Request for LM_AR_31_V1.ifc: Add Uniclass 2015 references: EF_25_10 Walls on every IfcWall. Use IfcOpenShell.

First a look at what the model holds.

```python
import ifcopenshell

model = ifcopenshell.open("LM_AR_31_V1.ifc")
print(model.schema)
print("classifications:", [c.Name for c in model.by_type("IfcClassification")])
for ifc_class in ("IfcDoor", "IfcRoof", "IfcStair", "IfcWall", "IfcWindow"):
    print(ifc_class, len(model.by_type(ifc_class)))
```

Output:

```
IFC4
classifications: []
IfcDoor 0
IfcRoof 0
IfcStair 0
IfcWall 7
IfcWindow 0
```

```python
import ifcopenshell
import ifcopenshell.api.classification

model = ifcopenshell.open("LM_AR_31_V1.ifc")

system = ifcopenshell.api.classification.add_classification(model, classification="Uniclass 2015")

codes = {
    "IfcWall": ("EF_25_10", "Walls"),
}
for ifc_class, (code, name) in codes.items():
    products = model.by_type(ifc_class)
    ifcopenshell.api.classification.add_reference(
        model, products=products, classification=system, identification=code, name=name
    )
    print(code, len(products))

model.write("LM_AR_31_V1_updated.ifc")
```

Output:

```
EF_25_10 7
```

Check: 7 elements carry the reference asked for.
